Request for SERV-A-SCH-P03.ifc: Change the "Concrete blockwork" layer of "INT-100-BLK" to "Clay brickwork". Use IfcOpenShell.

First a look at what the model holds.

```python
import ifcopenshell
import ifcopenshell.util.element

model = ifcopenshell.open("SERV-A-SCH-P03.ifc")
print(model.schema)
for layer_set in model.by_type("IfcMaterialLayerSet"):
    if layer_set.LayerSetName == "INT-100-BLK":
        for layer in layer_set.MaterialLayers:
            print(layer.id(), layer.Material and layer.Material.Name, layer.LayerThickness, sep=" | ")
        print(len(ifcopenshell.util.element.get_elements_by_material(model, layer_set)), "elements and types use it")
print(sorted(m.Name for m in model.by_type("IfcMaterial") if m.Name)[:60])
```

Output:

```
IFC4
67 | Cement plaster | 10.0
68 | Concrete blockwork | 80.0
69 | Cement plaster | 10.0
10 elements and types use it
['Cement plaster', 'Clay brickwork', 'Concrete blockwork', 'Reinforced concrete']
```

```python
import ifcopenshell
import ifcopenshell.api.material

model = ifcopenshell.open("SERV-A-SCH-P03.ifc")

layer_set = next(s for s in model.by_type("IfcMaterialLayerSet") if s.LayerSetName == "INT-100-BLK")
layer = next(l for l in layer_set.MaterialLayers if l.Material and l.Material.Name == "Concrete blockwork")
material = next(m for m in model.by_type("IfcMaterial") if m.Name == "Clay brickwork")

# Point this one layer at the other material; renaming the old one would change it everywhere.
ifcopenshell.api.material.edit_layer(model, layer=layer, attributes={"Name": material.Name}, material=material)

print([l.Material.Name if l.Material else None for l in layer_set.MaterialLayers])

model.write("SERV-A-SCH-P03_updated.ifc")
```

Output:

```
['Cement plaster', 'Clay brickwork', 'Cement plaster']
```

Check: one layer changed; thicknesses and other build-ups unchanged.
